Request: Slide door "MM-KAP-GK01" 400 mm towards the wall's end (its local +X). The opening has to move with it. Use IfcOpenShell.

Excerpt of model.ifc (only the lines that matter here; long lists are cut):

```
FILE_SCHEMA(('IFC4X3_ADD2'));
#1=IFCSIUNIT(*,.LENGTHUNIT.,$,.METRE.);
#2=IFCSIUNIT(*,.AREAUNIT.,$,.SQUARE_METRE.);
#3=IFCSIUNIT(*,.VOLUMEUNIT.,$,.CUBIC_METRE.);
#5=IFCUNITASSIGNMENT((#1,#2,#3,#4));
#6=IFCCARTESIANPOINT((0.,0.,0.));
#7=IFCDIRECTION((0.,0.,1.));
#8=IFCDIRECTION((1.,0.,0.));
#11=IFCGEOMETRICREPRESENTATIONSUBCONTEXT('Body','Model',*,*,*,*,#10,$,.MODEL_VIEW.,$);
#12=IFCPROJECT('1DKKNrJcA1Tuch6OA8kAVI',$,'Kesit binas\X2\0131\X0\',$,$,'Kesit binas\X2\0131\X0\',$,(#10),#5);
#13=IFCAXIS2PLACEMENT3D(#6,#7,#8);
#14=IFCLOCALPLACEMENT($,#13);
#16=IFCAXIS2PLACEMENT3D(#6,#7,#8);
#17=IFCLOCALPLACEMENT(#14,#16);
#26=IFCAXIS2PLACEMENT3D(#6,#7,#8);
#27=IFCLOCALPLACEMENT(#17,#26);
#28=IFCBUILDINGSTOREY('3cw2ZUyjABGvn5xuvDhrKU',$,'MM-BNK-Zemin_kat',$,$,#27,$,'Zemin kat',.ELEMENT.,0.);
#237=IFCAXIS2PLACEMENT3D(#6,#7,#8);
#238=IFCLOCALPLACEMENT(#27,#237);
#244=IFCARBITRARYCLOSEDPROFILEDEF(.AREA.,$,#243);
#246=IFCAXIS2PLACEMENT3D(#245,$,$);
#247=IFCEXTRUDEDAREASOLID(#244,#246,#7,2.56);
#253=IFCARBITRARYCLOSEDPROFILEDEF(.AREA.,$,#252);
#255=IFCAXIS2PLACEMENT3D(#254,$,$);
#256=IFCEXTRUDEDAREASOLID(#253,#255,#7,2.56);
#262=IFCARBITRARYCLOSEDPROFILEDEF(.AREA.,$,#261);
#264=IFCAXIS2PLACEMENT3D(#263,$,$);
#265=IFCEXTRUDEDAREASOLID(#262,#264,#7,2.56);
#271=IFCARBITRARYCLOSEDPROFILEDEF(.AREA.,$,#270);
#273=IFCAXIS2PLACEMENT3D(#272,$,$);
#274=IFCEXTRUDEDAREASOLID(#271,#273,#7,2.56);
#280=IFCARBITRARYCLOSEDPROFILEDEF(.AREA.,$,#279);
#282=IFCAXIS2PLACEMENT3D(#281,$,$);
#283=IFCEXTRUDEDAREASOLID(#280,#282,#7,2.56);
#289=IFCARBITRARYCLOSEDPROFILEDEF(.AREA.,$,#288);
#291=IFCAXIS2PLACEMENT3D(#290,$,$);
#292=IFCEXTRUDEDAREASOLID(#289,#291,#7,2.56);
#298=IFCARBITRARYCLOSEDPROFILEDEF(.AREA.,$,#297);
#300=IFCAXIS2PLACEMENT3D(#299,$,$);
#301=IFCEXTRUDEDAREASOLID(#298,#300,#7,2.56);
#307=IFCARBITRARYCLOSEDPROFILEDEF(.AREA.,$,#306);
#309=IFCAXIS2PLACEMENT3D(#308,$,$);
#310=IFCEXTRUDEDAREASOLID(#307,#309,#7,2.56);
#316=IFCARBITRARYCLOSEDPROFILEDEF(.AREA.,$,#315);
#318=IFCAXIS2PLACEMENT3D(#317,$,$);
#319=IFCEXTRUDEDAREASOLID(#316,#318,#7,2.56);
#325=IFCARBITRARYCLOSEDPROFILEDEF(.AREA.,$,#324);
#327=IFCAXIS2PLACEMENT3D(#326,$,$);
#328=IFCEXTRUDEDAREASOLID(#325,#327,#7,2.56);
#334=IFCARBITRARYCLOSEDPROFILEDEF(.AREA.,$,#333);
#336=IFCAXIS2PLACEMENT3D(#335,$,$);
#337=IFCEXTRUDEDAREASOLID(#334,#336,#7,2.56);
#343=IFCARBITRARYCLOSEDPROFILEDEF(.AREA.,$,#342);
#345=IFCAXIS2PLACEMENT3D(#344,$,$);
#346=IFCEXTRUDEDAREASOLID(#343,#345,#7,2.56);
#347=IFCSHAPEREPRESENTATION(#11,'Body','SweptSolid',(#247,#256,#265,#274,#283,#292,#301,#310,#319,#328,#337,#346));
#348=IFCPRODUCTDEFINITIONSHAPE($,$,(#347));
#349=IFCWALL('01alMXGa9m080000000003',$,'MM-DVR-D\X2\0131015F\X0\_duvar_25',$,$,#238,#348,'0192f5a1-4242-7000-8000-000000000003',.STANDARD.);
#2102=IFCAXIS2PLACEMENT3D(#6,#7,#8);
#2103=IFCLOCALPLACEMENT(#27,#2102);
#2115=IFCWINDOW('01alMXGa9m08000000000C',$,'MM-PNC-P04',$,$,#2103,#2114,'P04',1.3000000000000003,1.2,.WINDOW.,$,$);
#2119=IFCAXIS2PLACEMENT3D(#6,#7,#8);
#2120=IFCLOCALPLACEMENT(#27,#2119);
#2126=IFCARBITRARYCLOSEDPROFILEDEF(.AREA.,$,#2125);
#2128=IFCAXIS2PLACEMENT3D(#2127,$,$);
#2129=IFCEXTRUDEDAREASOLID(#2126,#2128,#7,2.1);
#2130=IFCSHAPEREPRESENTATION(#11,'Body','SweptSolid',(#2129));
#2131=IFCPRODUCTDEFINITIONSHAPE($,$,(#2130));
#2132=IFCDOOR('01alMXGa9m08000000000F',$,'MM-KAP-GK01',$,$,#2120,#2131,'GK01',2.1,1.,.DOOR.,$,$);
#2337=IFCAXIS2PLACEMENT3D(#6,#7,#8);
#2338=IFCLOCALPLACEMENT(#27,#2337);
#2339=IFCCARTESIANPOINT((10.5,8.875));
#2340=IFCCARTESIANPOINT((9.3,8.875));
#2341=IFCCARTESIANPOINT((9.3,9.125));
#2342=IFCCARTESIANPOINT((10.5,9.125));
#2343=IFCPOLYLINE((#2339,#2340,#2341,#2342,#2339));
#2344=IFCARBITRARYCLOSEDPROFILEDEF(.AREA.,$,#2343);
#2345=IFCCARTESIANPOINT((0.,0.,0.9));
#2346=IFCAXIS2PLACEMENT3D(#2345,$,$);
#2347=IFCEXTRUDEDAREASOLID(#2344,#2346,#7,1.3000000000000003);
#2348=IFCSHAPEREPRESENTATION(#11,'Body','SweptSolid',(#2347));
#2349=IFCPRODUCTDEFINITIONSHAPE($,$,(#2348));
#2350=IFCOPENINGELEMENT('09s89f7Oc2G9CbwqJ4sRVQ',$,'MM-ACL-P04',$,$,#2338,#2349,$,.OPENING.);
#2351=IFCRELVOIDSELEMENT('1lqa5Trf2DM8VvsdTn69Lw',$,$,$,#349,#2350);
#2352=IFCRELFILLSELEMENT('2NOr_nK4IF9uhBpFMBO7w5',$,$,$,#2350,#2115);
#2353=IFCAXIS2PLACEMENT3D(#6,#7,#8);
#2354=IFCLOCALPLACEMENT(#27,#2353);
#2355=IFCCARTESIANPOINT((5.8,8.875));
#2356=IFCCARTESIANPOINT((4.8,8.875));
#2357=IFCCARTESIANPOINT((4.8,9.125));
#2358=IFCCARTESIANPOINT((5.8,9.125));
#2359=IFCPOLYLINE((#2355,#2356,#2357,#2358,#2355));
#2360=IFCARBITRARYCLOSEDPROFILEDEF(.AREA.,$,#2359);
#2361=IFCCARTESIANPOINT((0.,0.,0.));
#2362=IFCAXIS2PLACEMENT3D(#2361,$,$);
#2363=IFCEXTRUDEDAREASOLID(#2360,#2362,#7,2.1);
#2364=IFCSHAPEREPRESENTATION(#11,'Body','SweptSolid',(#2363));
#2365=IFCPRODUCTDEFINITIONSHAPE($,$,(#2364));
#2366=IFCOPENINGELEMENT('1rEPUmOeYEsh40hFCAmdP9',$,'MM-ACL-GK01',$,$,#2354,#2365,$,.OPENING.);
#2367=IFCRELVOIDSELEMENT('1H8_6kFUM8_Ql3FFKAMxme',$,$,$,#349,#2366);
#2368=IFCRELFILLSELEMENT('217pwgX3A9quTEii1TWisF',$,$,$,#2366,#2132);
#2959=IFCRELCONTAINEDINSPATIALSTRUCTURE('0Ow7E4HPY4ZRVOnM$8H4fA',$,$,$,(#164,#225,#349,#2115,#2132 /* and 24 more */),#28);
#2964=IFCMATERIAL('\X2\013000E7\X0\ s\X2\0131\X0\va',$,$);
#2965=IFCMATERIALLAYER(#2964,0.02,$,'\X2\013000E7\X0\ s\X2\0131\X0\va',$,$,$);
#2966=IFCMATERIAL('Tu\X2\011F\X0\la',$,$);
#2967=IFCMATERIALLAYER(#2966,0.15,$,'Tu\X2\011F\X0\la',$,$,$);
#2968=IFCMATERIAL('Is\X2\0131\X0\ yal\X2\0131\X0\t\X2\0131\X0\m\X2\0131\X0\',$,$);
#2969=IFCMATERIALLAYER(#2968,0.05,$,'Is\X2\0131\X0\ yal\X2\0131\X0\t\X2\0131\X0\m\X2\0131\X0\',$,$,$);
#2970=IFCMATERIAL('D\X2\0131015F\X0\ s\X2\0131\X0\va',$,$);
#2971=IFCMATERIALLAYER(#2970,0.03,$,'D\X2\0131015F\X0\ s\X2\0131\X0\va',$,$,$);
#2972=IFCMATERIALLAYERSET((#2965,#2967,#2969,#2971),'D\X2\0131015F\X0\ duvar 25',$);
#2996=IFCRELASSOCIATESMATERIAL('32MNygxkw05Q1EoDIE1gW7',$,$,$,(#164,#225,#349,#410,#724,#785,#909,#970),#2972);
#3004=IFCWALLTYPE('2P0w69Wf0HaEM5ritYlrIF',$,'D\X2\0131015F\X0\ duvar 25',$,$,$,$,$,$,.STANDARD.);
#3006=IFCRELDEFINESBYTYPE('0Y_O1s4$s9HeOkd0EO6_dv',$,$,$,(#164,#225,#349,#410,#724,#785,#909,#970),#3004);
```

```python
import ifcopenshell
import ifcopenshell.api.geometry
import ifcopenshell.util.placement
import ifcopenshell.util.unit

model = ifcopenshell.open("model.ifc")
unit_scale = ifcopenshell.util.unit.calculate_unit_scale(model)

door = model.by_guid("01alMXGa9m08000000000F")
opening = door.FillsVoids[0].RelatingOpeningElement
wall = opening.VoidsElements[0].RelatingBuildingElement

wall_matrix = ifcopenshell.util.placement.get_local_placement(wall.ObjectPlacement)
shift = wall_matrix[:3, 0] * 0.4 / unit_scale
before = ifcopenshell.util.placement.get_local_placement(door.ObjectPlacement)[:3, 3].copy()

# The door is not placed relative to its opening, so move both.
for product in (opening, door):
    matrix = ifcopenshell.util.placement.get_local_placement(product.ObjectPlacement)
    matrix[:3, 3] += shift
    ifcopenshell.api.geometry.edit_object_placement(model, product=product, matrix=matrix, is_si=False)

after = ifcopenshell.util.placement.get_local_placement(door.ObjectPlacement)[:3, 3]
print("door moved by", (after - before).round(3) + 0.0)

model.write("model_updated.ifc")
```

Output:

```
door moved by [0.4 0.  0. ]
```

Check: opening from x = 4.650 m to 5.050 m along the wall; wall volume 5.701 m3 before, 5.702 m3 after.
